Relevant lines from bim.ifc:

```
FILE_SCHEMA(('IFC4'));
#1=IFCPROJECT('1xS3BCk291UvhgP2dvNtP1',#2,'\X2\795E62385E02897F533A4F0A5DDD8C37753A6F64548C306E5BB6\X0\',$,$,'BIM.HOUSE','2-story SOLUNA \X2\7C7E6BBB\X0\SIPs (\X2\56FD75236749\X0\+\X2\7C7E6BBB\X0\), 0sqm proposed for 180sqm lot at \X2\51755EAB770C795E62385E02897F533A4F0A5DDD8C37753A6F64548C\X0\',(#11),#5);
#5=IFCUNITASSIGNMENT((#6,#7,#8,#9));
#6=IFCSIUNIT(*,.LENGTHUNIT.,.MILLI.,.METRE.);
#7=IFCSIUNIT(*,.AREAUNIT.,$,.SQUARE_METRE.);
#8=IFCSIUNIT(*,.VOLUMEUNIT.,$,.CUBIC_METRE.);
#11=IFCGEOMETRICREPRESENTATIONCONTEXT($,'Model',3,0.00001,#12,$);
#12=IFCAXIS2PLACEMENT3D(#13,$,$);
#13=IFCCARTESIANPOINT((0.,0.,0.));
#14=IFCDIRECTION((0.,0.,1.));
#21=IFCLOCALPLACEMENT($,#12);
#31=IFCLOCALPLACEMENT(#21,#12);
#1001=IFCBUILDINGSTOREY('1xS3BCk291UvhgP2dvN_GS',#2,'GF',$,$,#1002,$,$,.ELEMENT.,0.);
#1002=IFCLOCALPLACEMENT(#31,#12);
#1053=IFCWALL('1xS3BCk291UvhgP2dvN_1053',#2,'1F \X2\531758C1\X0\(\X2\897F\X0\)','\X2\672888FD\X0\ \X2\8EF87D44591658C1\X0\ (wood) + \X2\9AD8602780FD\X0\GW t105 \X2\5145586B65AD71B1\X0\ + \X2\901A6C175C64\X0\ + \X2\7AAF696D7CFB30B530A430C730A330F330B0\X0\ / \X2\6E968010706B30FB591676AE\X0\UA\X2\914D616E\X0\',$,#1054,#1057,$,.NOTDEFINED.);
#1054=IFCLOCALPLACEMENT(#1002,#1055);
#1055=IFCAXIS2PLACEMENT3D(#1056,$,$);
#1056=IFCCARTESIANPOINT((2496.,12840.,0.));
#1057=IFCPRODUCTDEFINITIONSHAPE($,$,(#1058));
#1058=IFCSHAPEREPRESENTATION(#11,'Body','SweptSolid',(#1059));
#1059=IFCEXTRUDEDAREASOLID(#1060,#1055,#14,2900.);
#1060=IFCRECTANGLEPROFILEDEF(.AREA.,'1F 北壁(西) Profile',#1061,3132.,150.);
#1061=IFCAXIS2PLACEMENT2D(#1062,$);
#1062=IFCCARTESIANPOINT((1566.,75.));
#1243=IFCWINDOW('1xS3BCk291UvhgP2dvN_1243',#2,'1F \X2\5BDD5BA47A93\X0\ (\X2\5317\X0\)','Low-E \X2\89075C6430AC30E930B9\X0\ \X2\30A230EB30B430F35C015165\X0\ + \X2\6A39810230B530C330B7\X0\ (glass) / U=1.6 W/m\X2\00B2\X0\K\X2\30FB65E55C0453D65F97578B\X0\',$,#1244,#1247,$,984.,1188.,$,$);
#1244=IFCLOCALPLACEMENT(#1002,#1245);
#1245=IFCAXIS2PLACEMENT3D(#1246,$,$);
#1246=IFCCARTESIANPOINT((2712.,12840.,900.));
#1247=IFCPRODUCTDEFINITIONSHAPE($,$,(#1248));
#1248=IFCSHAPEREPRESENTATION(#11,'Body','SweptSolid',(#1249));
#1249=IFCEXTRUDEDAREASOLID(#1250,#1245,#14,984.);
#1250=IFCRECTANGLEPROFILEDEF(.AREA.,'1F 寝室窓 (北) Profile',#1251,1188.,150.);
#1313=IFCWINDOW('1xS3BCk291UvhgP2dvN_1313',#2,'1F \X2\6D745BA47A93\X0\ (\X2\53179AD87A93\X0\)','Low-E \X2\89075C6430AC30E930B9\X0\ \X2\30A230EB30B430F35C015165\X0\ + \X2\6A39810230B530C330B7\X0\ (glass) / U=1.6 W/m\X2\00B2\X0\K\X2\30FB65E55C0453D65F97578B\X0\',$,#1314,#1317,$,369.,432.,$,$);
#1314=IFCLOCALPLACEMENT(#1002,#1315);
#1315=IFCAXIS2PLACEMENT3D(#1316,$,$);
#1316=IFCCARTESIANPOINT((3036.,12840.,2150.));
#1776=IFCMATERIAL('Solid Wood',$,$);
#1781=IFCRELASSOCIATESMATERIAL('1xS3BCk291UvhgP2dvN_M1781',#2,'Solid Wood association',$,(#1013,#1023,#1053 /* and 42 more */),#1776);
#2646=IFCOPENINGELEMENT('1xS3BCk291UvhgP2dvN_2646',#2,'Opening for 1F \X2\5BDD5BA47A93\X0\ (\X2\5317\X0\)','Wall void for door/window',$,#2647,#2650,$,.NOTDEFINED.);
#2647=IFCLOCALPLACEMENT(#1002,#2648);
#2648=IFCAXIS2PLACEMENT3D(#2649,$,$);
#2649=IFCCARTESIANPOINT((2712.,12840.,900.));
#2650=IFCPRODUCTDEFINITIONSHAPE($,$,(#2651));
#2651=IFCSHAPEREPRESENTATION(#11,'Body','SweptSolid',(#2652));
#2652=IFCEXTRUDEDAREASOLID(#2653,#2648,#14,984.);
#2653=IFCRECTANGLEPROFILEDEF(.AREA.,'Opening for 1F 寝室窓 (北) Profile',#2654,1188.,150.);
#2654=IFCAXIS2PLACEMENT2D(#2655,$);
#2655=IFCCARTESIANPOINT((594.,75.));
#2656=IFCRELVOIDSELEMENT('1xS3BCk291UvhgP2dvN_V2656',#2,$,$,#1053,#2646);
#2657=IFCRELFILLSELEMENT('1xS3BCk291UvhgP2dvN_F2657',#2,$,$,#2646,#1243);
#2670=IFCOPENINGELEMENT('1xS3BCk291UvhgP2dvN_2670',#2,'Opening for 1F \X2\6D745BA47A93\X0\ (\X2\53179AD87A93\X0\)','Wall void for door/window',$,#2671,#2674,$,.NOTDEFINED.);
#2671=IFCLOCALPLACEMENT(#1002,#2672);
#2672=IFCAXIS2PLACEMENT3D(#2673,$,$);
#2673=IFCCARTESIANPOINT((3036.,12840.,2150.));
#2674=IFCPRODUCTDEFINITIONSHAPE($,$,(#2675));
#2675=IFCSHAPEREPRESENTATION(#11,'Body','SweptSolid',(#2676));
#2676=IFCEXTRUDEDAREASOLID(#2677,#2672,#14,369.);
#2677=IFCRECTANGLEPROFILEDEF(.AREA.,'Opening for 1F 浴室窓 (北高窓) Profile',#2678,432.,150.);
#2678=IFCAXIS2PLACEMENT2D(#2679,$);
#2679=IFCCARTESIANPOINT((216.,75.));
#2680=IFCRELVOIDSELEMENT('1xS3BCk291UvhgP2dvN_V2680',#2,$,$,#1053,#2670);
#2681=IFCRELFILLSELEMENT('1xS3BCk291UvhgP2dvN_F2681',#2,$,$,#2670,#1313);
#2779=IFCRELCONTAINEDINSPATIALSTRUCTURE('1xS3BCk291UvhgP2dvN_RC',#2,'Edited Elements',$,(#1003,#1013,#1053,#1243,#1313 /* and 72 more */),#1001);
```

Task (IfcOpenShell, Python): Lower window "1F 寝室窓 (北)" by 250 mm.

```python
import numpy as np
import ifcopenshell
import ifcopenshell.api.geometry
import ifcopenshell.util.placement
import ifcopenshell.util.unit

model = ifcopenshell.open("bim.ifc")
unit_scale = ifcopenshell.util.unit.calculate_unit_scale(model)

window = model.by_id(1243)
opening = window.FillsVoids[0].RelatingOpeningElement
dz = -0.25 / unit_scale

shift = np.array([0.0, 0.0, dz])
# The window is not placed relative to its opening, so move both.
for product in (opening, window):
    matrix = ifcopenshell.util.placement.get_local_placement(product.ObjectPlacement)
    matrix[:3, 3] += shift
    ifcopenshell.api.geometry.edit_object_placement(model, product=product, matrix=matrix, is_si=False)

print(f"moved by {dz * unit_scale:+.3f} m")

model.write("bim_updated.ifc")
```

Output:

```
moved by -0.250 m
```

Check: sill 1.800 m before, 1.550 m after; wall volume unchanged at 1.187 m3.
